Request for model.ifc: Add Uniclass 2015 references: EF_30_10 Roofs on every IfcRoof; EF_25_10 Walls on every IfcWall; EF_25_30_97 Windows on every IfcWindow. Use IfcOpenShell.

First a look at what the model holds.

```python
import ifcopenshell

model = ifcopenshell.open("model.ifc")
print(model.schema)
print("classifications:", [c.Name for c in model.by_type("IfcClassification")])
for ifc_class in ("IfcDoor", "IfcRoof", "IfcStair", "IfcWall", "IfcWindow"):
    print(ifc_class, len(model.by_type(ifc_class)))
```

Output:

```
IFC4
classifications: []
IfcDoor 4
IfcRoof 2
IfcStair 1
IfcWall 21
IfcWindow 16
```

```python
import ifcopenshell
import ifcopenshell.api.classification

model = ifcopenshell.open("model.ifc")

system = ifcopenshell.api.classification.add_classification(model, classification="Uniclass 2015")

codes = {
    "IfcRoof": ("EF_30_10", "Roofs"),
    "IfcWall": ("EF_25_10", "Walls"),
    "IfcWindow": ("EF_25_30_97", "Windows"),
}
for ifc_class, (code, name) in codes.items():
    products = model.by_type(ifc_class)
    ifcopenshell.api.classification.add_reference(
        model, products=products, classification=system, identification=code, name=name
    )
    print(code, len(products))

model.write("model_v2.ifc")
```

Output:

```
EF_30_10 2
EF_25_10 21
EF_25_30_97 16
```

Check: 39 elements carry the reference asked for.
